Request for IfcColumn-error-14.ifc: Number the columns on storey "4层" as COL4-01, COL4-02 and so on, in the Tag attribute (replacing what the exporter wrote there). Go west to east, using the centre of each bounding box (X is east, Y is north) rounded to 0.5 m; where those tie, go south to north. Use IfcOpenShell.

First a look at what the model holds.

```python
import ifcopenshell
import ifcopenshell.util.element
import ifcopenshell.util.placement

model = ifcopenshell.open("IfcColumn-error-14.ifc")
print(model.schema)
storey = next(s for s in model.by_type("IfcBuildingStorey") if s.Name == "4层")
columns = [e for e in ifcopenshell.util.element.get_decomposition(storey) if e.is_a("IfcColumn")]
for e in sorted(columns, key=lambda e: e.id()):
    origin = ifcopenshell.util.placement.get_local_placement(e.ObjectPlacement)[:3, 3]
    print(e.id(), e.Tag, e.Name, origin.round(2) + 0.0, sep=" | ")
```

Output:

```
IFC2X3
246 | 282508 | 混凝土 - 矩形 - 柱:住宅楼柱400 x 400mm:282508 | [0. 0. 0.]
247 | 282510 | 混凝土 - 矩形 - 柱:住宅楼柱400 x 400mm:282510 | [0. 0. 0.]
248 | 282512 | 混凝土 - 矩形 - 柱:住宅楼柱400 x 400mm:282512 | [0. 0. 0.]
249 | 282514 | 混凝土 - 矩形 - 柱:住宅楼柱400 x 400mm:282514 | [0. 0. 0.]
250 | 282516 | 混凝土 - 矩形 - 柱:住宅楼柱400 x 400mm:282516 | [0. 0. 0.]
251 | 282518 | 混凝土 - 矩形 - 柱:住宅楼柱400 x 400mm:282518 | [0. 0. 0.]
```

```python
import ifcopenshell
import ifcopenshell.geom
import ifcopenshell.util.element
import ifcopenshell.util.shape

model = ifcopenshell.open("IfcColumn-error-14.ifc")
settings = ifcopenshell.geom.settings()
settings.set("use-world-coords", True)


def centre(element):
    shape = ifcopenshell.geom.create_shape(settings, element)
    return ifcopenshell.util.shape.get_bbox_centroid(shape.geometry)


storey = next(s for s in model.by_type("IfcBuildingStorey") if s.Name == "4层")
columns = [e for e in ifcopenshell.util.element.get_decomposition(storey) if e.is_a("IfcColumn")]

# Insertion points can sit at a corner or the storey origin, so sort by the geometry (in metres).
centres = {e: centre(e) for e in columns}
columns.sort(key=lambda e: (round(centres[e][0] / 0.5), centres[e][1]))

for i, e in enumerate(columns, start=1):
    number = f"COL4-{i:02d}"
    e.Tag = number
    print(e.id(), number)

model.write("IfcColumn-error-14_rev.ifc")
```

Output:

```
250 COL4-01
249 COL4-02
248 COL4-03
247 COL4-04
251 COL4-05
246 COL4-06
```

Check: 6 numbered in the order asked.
